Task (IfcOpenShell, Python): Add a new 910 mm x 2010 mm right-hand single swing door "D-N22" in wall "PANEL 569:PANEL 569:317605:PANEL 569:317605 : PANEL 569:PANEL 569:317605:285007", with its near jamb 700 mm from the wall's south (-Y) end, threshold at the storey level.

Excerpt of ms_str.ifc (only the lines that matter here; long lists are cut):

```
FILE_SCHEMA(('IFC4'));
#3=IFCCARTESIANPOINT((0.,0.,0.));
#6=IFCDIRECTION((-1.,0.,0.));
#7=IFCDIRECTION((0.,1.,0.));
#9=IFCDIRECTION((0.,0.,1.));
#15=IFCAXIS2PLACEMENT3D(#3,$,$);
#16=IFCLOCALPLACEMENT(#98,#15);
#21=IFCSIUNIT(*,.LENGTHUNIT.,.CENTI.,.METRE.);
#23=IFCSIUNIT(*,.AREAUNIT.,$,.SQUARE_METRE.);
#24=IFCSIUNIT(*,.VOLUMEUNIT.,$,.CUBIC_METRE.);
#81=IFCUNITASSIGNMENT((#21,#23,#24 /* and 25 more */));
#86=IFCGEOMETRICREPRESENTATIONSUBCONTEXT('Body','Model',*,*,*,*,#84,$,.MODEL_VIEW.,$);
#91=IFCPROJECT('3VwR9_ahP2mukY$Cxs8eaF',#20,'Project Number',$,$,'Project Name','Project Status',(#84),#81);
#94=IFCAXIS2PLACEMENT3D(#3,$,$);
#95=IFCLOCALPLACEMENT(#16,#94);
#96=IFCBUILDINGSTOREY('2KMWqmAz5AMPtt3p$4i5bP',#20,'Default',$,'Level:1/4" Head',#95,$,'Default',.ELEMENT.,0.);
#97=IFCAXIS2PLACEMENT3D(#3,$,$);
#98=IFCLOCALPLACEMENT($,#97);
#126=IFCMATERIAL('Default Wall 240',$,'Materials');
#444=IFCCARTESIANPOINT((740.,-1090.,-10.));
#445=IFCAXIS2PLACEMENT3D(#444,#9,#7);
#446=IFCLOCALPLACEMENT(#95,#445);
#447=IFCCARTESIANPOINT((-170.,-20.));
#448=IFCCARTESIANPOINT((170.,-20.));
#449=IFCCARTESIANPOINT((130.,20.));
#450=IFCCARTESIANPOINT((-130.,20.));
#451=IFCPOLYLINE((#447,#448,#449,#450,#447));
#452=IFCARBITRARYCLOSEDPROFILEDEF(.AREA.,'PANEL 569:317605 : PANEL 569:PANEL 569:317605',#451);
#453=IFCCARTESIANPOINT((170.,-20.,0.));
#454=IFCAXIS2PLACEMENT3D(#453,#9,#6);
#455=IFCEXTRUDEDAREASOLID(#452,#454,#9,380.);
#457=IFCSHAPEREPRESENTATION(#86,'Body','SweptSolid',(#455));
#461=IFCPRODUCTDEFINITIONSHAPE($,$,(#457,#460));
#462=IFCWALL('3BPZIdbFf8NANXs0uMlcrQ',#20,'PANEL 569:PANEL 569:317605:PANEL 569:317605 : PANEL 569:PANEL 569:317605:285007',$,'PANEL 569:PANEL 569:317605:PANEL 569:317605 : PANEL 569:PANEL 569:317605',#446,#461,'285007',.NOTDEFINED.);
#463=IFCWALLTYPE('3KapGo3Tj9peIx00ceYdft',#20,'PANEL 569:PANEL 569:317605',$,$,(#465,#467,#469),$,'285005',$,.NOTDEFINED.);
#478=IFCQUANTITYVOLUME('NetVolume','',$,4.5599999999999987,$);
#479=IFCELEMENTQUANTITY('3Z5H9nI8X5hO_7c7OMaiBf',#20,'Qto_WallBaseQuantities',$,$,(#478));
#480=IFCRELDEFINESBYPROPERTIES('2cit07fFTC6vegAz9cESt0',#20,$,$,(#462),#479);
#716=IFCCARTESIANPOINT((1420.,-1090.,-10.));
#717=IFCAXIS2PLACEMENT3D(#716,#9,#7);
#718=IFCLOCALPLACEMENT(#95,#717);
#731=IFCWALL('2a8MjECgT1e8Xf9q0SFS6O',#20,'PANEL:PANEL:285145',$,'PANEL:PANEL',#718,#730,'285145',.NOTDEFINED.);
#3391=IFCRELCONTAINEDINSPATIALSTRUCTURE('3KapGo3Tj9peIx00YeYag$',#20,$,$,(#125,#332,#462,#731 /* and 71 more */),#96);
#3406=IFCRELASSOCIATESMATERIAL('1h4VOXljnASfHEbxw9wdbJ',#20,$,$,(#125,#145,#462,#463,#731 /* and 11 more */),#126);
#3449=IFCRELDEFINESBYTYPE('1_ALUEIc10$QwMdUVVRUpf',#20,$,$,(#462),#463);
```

```python
import numpy as np
import ifcopenshell
import ifcopenshell.api.feature
import ifcopenshell.api.geometry
import ifcopenshell.api.pset
import ifcopenshell.api.root
import ifcopenshell.api.spatial
import ifcopenshell.geom
import ifcopenshell.util.element
import ifcopenshell.util.placement
import ifcopenshell.util.representation
import ifcopenshell.util.shape
import ifcopenshell.util.unit

model = ifcopenshell.open("ms_str.ifc")
unit_scale = ifcopenshell.util.unit.calculate_unit_scale(model)
volume_scale = ifcopenshell.util.unit.calculate_unit_scale(model, "VOLUMEUNIT")
settings = ifcopenshell.geom.settings()


def volume(element):
    """Net volume in cubic metres, openings subtracted."""
    shape = ifcopenshell.geom.create_shape(settings, element)
    return ifcopenshell.util.shape.get_volume(shape.geometry)


wall = model.by_guid("3BPZIdbFf8NANXs0uMlcrQ")
storey = ifcopenshell.util.element.get_container(wall, ifc_class="IfcBuildingStorey")
context = ifcopenshell.util.representation.get_context(model, "Model", "Body", "MODEL_VIEW")
before = volume(wall)

width, height, from_end, sill = 0.91, 2.01, 0.7, 0.0  # metres

# The wall runs along its own X axis, and the end named is its -X end.
wall_shape = ifcopenshell.geom.create_shape(settings, wall)
x, y, z = ifcopenshell.util.shape.get_vertices(wall_shape.geometry).T
start = x.min() + from_end
face, thickness = float(y.min()), float(y.max() - y.min())
wall_matrix = ifcopenshell.util.placement.get_local_placement(wall.ObjectPlacement)
level = ifcopenshell.util.placement.get_local_placement(storey.ObjectPlacement)[2, 3]


def in_wall(x, y):
    """Placement at x, y metres in the wall's axes, at sill height."""
    matrix = wall_matrix.copy()
    matrix[:, 3] = wall_matrix @ np.array([x / unit_scale, y / unit_scale, 0.0, 1.0])
    matrix[2, 3] = level + sill / unit_scale
    return matrix


# Opening: a box that overshoots both wall faces by 50 mm.
opening = ifcopenshell.api.root.create_entity(model, ifc_class="IfcOpeningElement", predefined_type="OPENING")
box = ifcopenshell.api.geometry.add_wall_representation(
    model, context=context, length=width, height=height, thickness=thickness + 0.1
)
ifcopenshell.api.geometry.assign_representation(model, product=opening, representation=box)
ifcopenshell.api.geometry.edit_object_placement(model, product=opening, matrix=in_wall(start, face - 0.05), is_si=False)
ifcopenshell.api.feature.add_feature(model, feature=opening, element=wall)

door = ifcopenshell.api.root.create_entity(model, ifc_class="IfcDoor", name="D-N22", predefined_type="DOOR")
door.OverallWidth, door.OverallHeight = width / unit_scale, height / unit_scale
door.OperationType = "SINGLE_SWING_RIGHT"
body = ifcopenshell.api.geometry.add_door_representation(
    model,
    context=context,
    overall_width=door.OverallWidth,
    overall_height=door.OverallHeight,
    operation_type="SINGLE_SWING_RIGHT",
    lining_properties={"LiningDepth": thickness / unit_scale, "ThresholdDepth": thickness / unit_scale},
)
ifcopenshell.api.geometry.assign_representation(model, product=door, representation=body)
ifcopenshell.api.spatial.assign_container(model, products=[door], relating_structure=storey)
ifcopenshell.api.feature.add_filling(model, opening=opening, element=door)

# The lining spans the wall, so the door starts at the wall face.
ifcopenshell.api.geometry.edit_object_placement(model, product=door, matrix=in_wall(start, face), is_si=False)

after = volume(wall)

# Update the wall's stored quantities.
qto = model.by_id(ifcopenshell.util.element.get_pset(wall, "Qto_WallBaseQuantities", should_inherit=False)["id"])
ifcopenshell.api.pset.edit_qto(model, qto=qto, properties={"NetVolume": after / volume_scale})

print(f"wall volume {before:.3f} -> {after:.3f} m3")

model.write("ms_str-out.ifc")
```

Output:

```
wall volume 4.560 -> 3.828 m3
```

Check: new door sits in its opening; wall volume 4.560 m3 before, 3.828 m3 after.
